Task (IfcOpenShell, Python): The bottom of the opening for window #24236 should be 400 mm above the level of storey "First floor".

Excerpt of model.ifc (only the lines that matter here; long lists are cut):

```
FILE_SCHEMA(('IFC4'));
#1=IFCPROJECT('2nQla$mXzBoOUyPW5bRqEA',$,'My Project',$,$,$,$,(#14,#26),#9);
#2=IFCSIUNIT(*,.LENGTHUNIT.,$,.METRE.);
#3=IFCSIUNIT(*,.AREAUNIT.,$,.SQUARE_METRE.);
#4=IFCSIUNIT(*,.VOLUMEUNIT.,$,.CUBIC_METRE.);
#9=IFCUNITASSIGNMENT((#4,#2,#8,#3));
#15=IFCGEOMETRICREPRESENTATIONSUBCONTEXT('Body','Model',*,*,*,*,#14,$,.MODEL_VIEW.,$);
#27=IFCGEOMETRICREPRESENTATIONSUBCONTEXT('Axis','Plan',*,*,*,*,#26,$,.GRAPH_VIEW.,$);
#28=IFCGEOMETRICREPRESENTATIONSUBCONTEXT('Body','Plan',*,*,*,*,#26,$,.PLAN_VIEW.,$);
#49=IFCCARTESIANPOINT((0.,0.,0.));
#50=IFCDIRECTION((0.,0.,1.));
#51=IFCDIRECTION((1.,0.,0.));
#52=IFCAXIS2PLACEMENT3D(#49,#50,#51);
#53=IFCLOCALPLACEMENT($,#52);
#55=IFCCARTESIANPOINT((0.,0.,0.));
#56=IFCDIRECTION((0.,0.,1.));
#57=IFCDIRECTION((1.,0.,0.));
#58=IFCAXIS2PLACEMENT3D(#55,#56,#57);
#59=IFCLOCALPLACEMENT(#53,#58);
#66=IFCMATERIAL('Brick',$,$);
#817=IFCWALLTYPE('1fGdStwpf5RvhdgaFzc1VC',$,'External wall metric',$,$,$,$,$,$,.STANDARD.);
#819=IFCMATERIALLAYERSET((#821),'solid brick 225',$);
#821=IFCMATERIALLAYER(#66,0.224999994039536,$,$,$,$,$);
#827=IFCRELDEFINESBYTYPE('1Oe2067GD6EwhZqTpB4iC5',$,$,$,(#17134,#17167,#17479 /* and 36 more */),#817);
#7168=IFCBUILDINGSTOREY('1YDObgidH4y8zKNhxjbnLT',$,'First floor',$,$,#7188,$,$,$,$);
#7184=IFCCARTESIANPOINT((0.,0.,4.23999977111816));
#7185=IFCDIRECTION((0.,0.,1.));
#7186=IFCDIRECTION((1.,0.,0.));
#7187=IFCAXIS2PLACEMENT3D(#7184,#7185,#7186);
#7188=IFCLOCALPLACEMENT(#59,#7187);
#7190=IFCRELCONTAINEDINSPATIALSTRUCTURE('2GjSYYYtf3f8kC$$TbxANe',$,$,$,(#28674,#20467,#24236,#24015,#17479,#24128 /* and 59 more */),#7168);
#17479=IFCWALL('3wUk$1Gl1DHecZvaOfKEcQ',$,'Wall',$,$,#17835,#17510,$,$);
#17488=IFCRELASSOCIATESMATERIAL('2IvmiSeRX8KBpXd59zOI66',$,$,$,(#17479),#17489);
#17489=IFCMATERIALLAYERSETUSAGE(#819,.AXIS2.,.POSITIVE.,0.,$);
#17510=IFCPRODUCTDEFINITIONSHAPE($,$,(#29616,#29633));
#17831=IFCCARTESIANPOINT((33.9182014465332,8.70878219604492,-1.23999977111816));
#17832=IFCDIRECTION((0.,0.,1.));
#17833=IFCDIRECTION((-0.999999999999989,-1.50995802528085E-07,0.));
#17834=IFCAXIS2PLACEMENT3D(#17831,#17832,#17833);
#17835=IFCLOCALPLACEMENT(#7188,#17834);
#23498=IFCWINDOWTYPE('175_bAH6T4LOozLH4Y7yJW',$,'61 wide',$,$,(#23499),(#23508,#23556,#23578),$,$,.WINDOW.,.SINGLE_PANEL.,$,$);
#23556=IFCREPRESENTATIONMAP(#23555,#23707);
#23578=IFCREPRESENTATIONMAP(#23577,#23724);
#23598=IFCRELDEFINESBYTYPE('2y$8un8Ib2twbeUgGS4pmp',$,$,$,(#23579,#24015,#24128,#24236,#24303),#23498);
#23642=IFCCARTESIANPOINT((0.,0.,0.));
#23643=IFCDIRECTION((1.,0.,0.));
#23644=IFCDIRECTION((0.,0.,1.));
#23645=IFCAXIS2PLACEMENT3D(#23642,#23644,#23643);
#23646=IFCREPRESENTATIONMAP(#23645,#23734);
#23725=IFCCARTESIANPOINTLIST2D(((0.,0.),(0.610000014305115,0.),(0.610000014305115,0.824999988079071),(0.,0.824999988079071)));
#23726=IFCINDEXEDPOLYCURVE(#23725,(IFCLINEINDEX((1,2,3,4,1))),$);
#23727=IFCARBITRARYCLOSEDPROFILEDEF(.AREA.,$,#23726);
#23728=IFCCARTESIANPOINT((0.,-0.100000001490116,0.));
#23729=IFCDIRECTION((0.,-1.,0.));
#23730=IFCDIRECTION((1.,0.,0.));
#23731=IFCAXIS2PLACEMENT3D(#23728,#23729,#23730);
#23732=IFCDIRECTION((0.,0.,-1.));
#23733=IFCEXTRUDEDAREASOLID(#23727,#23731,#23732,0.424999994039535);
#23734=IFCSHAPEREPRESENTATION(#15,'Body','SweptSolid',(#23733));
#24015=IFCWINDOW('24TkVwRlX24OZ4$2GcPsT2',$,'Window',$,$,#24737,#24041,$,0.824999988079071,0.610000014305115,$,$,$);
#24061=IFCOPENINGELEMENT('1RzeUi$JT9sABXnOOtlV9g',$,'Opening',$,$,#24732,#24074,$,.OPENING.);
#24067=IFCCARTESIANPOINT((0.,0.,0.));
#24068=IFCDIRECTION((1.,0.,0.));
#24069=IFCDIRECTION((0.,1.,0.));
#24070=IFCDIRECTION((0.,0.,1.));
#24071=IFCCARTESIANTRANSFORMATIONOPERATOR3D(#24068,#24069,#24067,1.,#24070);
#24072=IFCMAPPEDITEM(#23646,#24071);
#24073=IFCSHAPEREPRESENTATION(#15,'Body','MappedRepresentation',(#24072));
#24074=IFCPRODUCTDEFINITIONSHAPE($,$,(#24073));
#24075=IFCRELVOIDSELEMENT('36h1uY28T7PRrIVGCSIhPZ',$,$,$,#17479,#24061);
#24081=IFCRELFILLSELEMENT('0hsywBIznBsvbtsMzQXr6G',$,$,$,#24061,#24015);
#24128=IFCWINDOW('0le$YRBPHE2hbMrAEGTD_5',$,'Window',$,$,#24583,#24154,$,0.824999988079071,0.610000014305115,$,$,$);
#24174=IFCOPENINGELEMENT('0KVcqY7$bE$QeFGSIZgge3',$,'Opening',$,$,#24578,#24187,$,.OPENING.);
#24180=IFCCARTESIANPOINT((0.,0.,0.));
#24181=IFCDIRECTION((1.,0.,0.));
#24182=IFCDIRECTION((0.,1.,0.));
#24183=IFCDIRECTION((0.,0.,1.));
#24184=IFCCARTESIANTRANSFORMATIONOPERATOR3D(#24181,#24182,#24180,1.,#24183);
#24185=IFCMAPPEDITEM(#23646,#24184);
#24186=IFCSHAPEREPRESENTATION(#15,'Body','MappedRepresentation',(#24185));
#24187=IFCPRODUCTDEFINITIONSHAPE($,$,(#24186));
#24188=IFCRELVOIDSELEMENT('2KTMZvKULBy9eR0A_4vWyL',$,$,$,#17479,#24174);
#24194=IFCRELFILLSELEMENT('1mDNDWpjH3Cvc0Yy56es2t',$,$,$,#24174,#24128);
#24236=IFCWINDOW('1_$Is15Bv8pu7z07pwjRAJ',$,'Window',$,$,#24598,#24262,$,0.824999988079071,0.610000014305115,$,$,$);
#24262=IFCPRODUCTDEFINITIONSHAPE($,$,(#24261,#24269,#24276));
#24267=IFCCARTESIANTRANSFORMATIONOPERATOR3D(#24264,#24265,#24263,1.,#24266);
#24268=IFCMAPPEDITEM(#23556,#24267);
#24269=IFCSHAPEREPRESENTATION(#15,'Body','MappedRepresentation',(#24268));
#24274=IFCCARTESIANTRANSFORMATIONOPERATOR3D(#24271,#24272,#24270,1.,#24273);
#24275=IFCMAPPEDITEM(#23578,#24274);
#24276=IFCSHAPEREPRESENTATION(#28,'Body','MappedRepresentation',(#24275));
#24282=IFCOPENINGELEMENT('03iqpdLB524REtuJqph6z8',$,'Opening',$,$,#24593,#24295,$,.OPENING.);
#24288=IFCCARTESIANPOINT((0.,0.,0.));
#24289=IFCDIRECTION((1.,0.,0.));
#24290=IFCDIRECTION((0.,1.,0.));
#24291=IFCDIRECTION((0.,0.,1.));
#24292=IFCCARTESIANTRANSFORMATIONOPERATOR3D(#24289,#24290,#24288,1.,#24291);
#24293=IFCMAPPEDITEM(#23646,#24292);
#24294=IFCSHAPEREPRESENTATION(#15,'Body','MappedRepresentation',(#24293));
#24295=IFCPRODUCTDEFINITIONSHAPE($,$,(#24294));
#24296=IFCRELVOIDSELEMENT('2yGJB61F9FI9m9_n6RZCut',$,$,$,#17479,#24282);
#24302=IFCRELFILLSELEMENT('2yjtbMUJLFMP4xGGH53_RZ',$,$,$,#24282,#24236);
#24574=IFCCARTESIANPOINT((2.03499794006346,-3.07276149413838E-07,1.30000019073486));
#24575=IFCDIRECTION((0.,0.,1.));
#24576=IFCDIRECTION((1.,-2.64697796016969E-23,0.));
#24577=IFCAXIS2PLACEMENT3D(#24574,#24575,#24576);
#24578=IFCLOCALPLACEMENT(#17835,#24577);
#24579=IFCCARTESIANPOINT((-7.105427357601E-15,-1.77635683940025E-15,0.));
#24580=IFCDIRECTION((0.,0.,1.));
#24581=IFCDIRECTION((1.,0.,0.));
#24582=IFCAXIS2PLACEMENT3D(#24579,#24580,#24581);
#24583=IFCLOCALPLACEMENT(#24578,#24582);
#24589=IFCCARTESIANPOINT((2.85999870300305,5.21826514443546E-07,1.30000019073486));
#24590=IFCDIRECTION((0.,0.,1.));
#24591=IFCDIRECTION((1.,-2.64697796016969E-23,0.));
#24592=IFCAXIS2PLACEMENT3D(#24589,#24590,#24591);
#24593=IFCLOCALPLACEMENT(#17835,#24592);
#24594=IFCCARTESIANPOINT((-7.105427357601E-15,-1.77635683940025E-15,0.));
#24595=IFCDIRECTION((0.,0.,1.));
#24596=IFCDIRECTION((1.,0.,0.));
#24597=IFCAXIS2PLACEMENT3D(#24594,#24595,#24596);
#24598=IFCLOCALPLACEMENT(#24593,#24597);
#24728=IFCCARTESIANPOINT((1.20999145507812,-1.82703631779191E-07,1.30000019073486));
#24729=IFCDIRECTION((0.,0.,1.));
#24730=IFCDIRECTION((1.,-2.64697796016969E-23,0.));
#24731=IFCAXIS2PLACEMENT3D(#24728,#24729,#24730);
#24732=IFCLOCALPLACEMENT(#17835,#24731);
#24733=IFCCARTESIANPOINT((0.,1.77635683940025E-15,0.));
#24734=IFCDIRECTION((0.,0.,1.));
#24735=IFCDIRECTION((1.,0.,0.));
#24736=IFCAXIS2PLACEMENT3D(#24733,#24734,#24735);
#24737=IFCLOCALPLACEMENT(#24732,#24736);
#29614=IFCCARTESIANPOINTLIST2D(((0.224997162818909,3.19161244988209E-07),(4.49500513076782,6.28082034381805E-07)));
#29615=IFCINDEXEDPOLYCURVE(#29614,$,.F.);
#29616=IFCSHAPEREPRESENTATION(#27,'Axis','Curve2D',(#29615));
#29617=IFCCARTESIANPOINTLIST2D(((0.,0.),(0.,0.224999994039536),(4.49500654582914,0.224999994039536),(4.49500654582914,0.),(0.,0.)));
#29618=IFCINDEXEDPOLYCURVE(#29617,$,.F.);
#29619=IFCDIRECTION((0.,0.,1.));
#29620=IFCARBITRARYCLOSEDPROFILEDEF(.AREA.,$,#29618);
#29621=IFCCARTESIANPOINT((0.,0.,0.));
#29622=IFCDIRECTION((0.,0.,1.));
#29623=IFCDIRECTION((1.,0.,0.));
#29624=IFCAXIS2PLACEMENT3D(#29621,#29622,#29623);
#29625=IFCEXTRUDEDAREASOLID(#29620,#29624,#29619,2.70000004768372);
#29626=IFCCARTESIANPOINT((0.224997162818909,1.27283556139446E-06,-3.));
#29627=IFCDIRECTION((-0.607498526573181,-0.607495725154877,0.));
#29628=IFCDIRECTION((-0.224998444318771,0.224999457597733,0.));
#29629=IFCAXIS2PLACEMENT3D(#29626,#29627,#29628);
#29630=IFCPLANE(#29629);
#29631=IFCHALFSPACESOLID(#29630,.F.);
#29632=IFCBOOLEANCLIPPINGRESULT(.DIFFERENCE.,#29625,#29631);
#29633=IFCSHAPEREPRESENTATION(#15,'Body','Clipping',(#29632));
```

```python
import numpy as np
import ifcopenshell
import ifcopenshell.api.geometry
import ifcopenshell.geom
import ifcopenshell.util.element
import ifcopenshell.util.placement
import ifcopenshell.util.shape
import ifcopenshell.util.unit

model = ifcopenshell.open("model.ifc")
unit_scale = ifcopenshell.util.unit.calculate_unit_scale(model)

window = model.by_id(24236)
opening = window.FillsVoids[0].RelatingOpeningElement
storey = ifcopenshell.util.element.get_container(window, ifc_class="IfcBuildingStorey")
level = ifcopenshell.util.placement.get_local_placement(storey.ObjectPlacement)[2, 3]

# The opening's origin need not be at the sill, so measure its lowest point.
shape = ifcopenshell.geom.create_shape(ifcopenshell.geom.settings(), opening)
bottom = ifcopenshell.util.shape.get_shape_bottom_elevation(shape, shape.geometry) / unit_scale
dz = level + 0.4 / unit_scale - bottom

shift = np.array([0.0, 0.0, dz])
# The window is placed relative to its opening, so it follows when the opening moves.
matrix = ifcopenshell.util.placement.get_local_placement(opening.ObjectPlacement)
matrix[:3, 3] += shift
ifcopenshell.api.geometry.edit_object_placement(
    model, product=opening, matrix=matrix, is_si=False, should_transform_children=True
)

print(f"moved by {dz * unit_scale:+.3f} m")

model.write("model_edited.ifc")
```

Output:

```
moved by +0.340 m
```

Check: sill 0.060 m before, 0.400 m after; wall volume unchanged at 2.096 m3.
